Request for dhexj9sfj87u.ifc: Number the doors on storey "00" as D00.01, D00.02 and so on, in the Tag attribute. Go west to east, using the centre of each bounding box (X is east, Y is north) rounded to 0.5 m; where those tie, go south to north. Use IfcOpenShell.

First a look at what the model holds.

```python
import ifcopenshell
import ifcopenshell.util.element
import ifcopenshell.util.placement

model = ifcopenshell.open("dhexj9sfj87u.ifc")
print(model.schema)
storey = next(s for s in model.by_type("IfcBuildingStorey") if s.Name == "00")
doors = [e for e in ifcopenshell.util.element.get_decomposition(storey) if e.is_a("IfcDoor")]
for e in sorted(doors, key=lambda e: e.id()):
    origin = ifcopenshell.util.placement.get_local_placement(e.ObjectPlacement)[:3, 3]
    print(e.id(), e.Tag, e.Name, origin.round(2) + 0.0, sep=" | ")
```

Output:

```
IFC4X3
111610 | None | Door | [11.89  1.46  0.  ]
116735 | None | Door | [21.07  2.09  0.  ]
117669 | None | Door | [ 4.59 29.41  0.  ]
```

```python
import ifcopenshell
import ifcopenshell.geom
import ifcopenshell.util.element
import ifcopenshell.util.shape

model = ifcopenshell.open("dhexj9sfj87u.ifc")
settings = ifcopenshell.geom.settings()
settings.set("use-world-coords", True)


def centre(element):
    shape = ifcopenshell.geom.create_shape(settings, element)
    return ifcopenshell.util.shape.get_bbox_centroid(shape.geometry)


storey = next(s for s in model.by_type("IfcBuildingStorey") if s.Name == "00")
doors = [e for e in ifcopenshell.util.element.get_decomposition(storey) if e.is_a("IfcDoor")]

# Insertion points can sit at a corner or the storey origin, so sort by the geometry (in metres).
centres = {e: centre(e) for e in doors}
doors.sort(key=lambda e: (round(centres[e][0] / 0.5), centres[e][1]))

for i, e in enumerate(doors, start=1):
    number = f"D00.{i:02d}"
    e.Tag = number
    print(e.id(), number)

model.write("dhexj9sfj87u_updated.ifc")
```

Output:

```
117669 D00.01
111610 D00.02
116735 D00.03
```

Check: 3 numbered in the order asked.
